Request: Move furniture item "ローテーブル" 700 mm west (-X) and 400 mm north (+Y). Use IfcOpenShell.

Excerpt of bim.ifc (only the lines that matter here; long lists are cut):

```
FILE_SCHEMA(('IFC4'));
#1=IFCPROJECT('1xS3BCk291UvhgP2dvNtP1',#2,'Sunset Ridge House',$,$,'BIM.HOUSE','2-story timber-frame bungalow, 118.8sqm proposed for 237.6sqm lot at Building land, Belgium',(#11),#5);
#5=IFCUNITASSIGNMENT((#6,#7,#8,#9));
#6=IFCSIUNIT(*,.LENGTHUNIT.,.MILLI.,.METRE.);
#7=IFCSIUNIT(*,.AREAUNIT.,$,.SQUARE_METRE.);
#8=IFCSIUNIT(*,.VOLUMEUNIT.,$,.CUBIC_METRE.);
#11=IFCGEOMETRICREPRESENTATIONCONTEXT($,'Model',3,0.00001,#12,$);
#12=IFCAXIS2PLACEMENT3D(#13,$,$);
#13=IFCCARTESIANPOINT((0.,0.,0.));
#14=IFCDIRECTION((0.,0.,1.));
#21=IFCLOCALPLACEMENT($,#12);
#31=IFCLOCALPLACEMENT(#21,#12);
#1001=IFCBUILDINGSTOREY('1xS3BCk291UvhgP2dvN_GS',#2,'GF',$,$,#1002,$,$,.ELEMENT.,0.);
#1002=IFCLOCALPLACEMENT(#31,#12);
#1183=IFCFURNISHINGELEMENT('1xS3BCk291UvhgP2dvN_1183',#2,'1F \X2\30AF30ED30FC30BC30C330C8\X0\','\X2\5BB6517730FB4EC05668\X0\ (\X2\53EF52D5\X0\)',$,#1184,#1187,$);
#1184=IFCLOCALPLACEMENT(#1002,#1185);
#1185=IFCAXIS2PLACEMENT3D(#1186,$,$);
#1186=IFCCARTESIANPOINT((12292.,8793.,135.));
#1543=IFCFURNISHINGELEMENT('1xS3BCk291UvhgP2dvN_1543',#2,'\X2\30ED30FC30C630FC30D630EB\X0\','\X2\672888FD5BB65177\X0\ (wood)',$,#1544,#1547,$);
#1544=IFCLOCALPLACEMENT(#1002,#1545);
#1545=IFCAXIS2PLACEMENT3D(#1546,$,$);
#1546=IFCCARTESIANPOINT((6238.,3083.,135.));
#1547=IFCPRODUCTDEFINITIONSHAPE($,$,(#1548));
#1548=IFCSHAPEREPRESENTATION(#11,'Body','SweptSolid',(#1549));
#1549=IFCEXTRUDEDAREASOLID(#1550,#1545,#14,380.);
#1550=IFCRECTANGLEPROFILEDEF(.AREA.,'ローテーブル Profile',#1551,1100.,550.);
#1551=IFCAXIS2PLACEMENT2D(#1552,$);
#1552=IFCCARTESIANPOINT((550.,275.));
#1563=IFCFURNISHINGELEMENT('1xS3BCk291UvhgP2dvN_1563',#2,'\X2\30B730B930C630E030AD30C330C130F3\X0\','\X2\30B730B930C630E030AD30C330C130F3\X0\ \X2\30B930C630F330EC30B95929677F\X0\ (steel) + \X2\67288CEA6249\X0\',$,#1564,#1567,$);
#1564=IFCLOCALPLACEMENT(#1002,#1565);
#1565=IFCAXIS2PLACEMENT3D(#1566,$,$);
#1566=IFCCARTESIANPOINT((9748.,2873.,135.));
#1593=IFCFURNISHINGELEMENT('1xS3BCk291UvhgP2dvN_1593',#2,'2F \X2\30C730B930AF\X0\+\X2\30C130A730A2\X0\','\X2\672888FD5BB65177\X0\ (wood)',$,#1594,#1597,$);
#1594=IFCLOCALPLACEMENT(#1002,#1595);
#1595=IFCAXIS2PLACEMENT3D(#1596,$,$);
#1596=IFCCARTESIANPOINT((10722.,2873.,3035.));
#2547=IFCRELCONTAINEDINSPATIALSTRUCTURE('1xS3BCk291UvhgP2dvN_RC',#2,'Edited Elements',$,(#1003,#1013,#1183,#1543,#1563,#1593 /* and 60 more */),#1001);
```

```python
import ifcopenshell
import ifcopenshell.api.geometry
import ifcopenshell.util.placement

model = ifcopenshell.open("bim.ifc")

item = model.by_id(1543)
matrix = ifcopenshell.util.placement.get_local_placement(item.ObjectPlacement)
matrix[0, 3] -= 700.0
matrix[1, 3] += 400.0
ifcopenshell.api.geometry.edit_object_placement(model, product=item, matrix=matrix, is_si=False)

print(ifcopenshell.util.placement.get_local_placement(item.ObjectPlacement).round(3) + 0.0)

model.write("bim_edited.ifc")
```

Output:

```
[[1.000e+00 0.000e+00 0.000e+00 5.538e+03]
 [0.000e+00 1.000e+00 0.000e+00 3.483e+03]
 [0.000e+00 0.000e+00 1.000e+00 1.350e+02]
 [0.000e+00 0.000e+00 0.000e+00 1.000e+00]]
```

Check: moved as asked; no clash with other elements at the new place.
